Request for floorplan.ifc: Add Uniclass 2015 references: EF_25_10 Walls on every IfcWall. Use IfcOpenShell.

First a look at what the model holds.

```python
import ifcopenshell

model = ifcopenshell.open("floorplan.ifc")
print(model.schema)
print("classifications:", [c.Name for c in model.by_type("IfcClassification")])
for ifc_class in ("IfcDoor", "IfcRoof", "IfcStair", "IfcWall", "IfcWindow"):
    print(ifc_class, len(model.by_type(ifc_class)))
```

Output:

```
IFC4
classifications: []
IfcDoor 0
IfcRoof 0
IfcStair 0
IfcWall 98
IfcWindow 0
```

```python
import ifcopenshell
import ifcopenshell.api.classification

model = ifcopenshell.open("floorplan.ifc")

system = ifcopenshell.api.classification.add_classification(model, classification="Uniclass 2015")

codes = {
    "IfcWall": ("EF_25_10", "Walls"),
}
for ifc_class, (code, name) in codes.items():
    products = model.by_type(ifc_class)
    ifcopenshell.api.classification.add_reference(
        model, products=products, classification=system, identification=code, name=name
    )
    print(code, len(products))

model.write("floorplan_edited.ifc")
```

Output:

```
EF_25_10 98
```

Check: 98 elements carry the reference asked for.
